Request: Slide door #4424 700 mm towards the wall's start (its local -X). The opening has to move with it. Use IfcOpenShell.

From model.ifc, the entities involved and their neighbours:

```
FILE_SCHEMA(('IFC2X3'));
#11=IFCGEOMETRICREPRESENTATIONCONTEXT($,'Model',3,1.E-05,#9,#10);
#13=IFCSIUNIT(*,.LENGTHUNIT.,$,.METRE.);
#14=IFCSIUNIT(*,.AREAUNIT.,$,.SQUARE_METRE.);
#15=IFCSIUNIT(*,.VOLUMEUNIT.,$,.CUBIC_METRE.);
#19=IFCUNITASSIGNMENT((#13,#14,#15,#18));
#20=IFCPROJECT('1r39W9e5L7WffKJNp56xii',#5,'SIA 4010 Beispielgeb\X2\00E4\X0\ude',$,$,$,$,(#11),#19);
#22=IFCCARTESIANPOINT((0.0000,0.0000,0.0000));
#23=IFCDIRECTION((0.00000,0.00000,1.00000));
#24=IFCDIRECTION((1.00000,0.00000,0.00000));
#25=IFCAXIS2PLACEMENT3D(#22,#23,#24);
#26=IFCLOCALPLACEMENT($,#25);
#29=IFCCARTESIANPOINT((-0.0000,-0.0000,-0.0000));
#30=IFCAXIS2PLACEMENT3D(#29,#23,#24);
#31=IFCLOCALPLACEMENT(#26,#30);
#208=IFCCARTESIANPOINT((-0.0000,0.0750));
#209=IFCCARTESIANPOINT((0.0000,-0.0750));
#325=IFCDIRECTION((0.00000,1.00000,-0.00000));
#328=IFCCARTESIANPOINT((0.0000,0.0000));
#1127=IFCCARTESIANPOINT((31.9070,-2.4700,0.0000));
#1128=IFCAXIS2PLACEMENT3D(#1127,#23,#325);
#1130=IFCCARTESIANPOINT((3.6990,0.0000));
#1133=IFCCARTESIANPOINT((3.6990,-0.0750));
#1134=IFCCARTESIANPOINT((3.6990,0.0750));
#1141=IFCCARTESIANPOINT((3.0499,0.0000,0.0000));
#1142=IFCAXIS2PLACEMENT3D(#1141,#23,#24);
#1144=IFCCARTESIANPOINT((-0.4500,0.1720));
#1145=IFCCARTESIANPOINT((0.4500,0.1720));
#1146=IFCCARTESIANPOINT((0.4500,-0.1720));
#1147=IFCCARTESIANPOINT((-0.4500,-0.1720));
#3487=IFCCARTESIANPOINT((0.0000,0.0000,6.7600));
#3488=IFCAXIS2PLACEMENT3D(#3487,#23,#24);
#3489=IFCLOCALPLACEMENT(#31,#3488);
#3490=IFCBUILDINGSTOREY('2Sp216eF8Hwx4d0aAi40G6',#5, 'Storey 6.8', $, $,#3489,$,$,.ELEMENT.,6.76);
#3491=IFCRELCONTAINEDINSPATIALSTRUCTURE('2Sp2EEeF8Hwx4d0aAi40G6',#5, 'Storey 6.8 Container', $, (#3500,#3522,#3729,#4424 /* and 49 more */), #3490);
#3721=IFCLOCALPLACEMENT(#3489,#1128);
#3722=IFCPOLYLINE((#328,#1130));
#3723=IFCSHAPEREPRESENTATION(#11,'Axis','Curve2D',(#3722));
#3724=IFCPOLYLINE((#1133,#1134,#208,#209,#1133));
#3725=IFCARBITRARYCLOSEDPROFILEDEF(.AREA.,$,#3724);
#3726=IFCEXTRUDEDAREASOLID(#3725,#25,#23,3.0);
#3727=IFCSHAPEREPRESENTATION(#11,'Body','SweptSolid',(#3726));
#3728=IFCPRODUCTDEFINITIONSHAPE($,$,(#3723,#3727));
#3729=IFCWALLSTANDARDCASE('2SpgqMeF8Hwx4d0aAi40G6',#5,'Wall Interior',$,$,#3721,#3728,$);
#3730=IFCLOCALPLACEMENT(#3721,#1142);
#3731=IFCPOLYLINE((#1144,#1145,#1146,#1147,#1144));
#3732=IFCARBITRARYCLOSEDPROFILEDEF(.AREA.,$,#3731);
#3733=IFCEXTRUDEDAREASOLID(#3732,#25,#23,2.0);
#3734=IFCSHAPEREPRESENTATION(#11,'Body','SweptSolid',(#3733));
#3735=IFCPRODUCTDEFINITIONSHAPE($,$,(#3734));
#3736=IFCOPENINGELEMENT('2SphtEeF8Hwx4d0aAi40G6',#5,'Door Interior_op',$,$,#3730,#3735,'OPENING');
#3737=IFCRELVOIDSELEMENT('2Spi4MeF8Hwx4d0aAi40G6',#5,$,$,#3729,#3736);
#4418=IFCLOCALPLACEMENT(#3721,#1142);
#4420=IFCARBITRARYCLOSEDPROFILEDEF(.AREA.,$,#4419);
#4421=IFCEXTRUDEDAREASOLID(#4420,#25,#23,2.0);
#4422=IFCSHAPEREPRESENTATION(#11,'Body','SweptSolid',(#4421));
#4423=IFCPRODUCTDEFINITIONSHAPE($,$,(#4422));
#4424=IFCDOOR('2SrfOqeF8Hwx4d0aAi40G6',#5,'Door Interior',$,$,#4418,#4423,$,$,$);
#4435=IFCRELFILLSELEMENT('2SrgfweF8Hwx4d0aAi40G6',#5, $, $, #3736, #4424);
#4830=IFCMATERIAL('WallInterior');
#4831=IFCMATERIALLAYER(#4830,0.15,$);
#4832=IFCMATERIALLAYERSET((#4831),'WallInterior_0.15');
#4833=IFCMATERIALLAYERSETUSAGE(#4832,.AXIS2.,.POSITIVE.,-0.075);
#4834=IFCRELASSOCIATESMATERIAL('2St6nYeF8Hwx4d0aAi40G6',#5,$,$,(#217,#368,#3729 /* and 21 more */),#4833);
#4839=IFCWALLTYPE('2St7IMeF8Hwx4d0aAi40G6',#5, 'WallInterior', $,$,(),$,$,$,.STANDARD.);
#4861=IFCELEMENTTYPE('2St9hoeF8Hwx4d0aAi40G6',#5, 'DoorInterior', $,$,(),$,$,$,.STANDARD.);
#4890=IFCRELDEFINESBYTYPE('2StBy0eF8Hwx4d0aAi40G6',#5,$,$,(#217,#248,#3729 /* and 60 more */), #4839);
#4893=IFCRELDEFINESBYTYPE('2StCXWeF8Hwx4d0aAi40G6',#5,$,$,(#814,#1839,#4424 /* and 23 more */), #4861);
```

```python
import ifcopenshell
import ifcopenshell.api.geometry
import ifcopenshell.util.placement

model = ifcopenshell.open("model.ifc")

door = model.by_id(4424)
opening = door.FillsVoids[0].RelatingOpeningElement
wall = opening.VoidsElements[0].RelatingBuildingElement

wall_matrix = ifcopenshell.util.placement.get_local_placement(wall.ObjectPlacement)
shift = wall_matrix[:3, 0] * -0.7
before = ifcopenshell.util.placement.get_local_placement(door.ObjectPlacement)[:3, 3].copy()

# The door is not placed relative to its opening, so move both.
for product in (opening, door):
    matrix = ifcopenshell.util.placement.get_local_placement(product.ObjectPlacement)
    matrix[:3, 3] += shift
    ifcopenshell.api.geometry.edit_object_placement(model, product=product, matrix=matrix, is_si=False)

after = ifcopenshell.util.placement.get_local_placement(door.ObjectPlacement)[:3, 3]
print("door moved by", (after - before).round(3) + 0.0)

model.write("model_updated.ifc")
```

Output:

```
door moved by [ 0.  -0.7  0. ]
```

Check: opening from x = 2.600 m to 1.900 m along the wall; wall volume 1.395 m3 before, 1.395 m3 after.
